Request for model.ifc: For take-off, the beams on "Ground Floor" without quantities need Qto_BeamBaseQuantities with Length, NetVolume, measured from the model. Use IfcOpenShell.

First a look at what the model holds.

```python
import ifcopenshell
import ifcopenshell.util.element
import ifcopenshell.util.unit

model = ifcopenshell.open("model.ifc")
print(model.schema)
for unit_type in ("LENGTHUNIT", "AREAUNIT", "VOLUMEUNIT"):
    print(unit_type, ifcopenshell.util.unit.calculate_unit_scale(model, unit_type))
storey = next(s for s in model.by_type("IfcBuildingStorey") if s.Name == "Ground Floor")
beams = [e for e in ifcopenshell.util.element.get_decomposition(storey) if e.is_a("IfcBeam")]
for e in sorted(beams, key=lambda e: e.id()):
    print(e.id(), e.is_a(), e.Name, list(ifcopenshell.util.element.get_psets(e, qtos_only=True)), sep=" | ")
```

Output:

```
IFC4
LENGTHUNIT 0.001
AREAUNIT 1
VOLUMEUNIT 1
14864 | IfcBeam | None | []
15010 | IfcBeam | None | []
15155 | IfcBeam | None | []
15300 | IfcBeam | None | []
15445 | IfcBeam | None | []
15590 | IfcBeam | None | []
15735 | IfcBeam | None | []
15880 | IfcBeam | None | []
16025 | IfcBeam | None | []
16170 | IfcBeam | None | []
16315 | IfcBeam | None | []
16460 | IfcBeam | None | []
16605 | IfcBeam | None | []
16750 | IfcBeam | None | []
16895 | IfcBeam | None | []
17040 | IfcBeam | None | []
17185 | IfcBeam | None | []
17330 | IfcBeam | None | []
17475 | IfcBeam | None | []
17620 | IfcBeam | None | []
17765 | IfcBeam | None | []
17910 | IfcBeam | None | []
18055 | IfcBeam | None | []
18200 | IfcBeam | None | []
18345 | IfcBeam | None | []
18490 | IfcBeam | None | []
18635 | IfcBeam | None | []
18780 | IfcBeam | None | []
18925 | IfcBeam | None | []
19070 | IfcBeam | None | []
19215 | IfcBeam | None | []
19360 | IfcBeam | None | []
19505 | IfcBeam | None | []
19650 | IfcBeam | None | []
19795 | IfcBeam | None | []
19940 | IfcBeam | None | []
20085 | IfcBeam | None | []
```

```python
import ifcopenshell
import ifcopenshell.api.pset
import ifcopenshell.geom
import ifcopenshell.util.element
import ifcopenshell.util.shape
import ifcopenshell.util.unit

model = ifcopenshell.open("model.ifc")
unit_scale = ifcopenshell.util.unit.calculate_unit_scale(model)
volume_scale = ifcopenshell.util.unit.calculate_unit_scale(model, "VOLUMEUNIT")
settings = ifcopenshell.geom.settings()

storey = next(s for s in model.by_type("IfcBuildingStorey") if s.Name == "Ground Floor")
beams = [e for e in ifcopenshell.util.element.get_decomposition(storey) if e.is_a("IfcBeam")]

for e in sorted(beams, key=lambda e: e.id()):
    if ifcopenshell.util.element.get_psets(e, qtos_only=True, should_inherit=False):
        continue
    # Geometry comes back in metres, in the element's own axes.
    shape = ifcopenshell.geom.create_shape(settings, e)
    values = {
        "Length": ifcopenshell.util.shape.get_max_xyz(shape.geometry) / unit_scale,
        "NetVolume": ifcopenshell.util.shape.get_volume(shape.geometry) / volume_scale,
    }
    qto = ifcopenshell.api.pset.add_qto(model, product=e, name="Qto_BeamBaseQuantities")
    ifcopenshell.api.pset.edit_qto(model, qto=qto, properties=values)
    print(e.id(), {k: round(v, 3) for k, v in values.items()})

model.write("model_updated.ifc")
```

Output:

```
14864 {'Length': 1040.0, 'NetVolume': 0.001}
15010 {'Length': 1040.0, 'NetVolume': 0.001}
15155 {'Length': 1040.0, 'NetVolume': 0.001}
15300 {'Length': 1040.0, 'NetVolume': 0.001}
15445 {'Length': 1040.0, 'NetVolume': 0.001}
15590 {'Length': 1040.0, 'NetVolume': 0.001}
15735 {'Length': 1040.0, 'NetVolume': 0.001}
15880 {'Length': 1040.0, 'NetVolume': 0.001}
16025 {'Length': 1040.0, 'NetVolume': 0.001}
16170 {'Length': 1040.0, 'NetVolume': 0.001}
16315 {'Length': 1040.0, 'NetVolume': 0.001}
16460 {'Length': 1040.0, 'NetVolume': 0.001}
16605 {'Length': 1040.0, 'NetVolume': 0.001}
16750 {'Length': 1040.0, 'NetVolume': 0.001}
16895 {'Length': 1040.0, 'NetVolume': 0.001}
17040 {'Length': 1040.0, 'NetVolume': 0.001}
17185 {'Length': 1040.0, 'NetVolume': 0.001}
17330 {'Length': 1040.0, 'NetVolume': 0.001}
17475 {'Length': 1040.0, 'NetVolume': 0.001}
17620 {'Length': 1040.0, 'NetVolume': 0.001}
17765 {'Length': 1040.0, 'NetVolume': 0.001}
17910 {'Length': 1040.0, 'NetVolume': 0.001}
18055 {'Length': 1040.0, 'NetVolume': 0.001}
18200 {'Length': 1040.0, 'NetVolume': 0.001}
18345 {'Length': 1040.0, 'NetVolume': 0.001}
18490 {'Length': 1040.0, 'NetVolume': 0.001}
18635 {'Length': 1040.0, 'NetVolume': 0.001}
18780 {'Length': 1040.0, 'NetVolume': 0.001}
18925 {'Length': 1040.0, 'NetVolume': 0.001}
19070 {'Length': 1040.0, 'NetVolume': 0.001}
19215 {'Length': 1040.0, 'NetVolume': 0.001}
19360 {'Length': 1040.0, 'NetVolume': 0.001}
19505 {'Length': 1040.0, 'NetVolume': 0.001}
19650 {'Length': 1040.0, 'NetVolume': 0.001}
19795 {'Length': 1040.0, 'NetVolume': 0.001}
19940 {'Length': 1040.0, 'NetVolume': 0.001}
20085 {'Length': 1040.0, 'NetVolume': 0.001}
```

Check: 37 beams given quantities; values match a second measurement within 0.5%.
